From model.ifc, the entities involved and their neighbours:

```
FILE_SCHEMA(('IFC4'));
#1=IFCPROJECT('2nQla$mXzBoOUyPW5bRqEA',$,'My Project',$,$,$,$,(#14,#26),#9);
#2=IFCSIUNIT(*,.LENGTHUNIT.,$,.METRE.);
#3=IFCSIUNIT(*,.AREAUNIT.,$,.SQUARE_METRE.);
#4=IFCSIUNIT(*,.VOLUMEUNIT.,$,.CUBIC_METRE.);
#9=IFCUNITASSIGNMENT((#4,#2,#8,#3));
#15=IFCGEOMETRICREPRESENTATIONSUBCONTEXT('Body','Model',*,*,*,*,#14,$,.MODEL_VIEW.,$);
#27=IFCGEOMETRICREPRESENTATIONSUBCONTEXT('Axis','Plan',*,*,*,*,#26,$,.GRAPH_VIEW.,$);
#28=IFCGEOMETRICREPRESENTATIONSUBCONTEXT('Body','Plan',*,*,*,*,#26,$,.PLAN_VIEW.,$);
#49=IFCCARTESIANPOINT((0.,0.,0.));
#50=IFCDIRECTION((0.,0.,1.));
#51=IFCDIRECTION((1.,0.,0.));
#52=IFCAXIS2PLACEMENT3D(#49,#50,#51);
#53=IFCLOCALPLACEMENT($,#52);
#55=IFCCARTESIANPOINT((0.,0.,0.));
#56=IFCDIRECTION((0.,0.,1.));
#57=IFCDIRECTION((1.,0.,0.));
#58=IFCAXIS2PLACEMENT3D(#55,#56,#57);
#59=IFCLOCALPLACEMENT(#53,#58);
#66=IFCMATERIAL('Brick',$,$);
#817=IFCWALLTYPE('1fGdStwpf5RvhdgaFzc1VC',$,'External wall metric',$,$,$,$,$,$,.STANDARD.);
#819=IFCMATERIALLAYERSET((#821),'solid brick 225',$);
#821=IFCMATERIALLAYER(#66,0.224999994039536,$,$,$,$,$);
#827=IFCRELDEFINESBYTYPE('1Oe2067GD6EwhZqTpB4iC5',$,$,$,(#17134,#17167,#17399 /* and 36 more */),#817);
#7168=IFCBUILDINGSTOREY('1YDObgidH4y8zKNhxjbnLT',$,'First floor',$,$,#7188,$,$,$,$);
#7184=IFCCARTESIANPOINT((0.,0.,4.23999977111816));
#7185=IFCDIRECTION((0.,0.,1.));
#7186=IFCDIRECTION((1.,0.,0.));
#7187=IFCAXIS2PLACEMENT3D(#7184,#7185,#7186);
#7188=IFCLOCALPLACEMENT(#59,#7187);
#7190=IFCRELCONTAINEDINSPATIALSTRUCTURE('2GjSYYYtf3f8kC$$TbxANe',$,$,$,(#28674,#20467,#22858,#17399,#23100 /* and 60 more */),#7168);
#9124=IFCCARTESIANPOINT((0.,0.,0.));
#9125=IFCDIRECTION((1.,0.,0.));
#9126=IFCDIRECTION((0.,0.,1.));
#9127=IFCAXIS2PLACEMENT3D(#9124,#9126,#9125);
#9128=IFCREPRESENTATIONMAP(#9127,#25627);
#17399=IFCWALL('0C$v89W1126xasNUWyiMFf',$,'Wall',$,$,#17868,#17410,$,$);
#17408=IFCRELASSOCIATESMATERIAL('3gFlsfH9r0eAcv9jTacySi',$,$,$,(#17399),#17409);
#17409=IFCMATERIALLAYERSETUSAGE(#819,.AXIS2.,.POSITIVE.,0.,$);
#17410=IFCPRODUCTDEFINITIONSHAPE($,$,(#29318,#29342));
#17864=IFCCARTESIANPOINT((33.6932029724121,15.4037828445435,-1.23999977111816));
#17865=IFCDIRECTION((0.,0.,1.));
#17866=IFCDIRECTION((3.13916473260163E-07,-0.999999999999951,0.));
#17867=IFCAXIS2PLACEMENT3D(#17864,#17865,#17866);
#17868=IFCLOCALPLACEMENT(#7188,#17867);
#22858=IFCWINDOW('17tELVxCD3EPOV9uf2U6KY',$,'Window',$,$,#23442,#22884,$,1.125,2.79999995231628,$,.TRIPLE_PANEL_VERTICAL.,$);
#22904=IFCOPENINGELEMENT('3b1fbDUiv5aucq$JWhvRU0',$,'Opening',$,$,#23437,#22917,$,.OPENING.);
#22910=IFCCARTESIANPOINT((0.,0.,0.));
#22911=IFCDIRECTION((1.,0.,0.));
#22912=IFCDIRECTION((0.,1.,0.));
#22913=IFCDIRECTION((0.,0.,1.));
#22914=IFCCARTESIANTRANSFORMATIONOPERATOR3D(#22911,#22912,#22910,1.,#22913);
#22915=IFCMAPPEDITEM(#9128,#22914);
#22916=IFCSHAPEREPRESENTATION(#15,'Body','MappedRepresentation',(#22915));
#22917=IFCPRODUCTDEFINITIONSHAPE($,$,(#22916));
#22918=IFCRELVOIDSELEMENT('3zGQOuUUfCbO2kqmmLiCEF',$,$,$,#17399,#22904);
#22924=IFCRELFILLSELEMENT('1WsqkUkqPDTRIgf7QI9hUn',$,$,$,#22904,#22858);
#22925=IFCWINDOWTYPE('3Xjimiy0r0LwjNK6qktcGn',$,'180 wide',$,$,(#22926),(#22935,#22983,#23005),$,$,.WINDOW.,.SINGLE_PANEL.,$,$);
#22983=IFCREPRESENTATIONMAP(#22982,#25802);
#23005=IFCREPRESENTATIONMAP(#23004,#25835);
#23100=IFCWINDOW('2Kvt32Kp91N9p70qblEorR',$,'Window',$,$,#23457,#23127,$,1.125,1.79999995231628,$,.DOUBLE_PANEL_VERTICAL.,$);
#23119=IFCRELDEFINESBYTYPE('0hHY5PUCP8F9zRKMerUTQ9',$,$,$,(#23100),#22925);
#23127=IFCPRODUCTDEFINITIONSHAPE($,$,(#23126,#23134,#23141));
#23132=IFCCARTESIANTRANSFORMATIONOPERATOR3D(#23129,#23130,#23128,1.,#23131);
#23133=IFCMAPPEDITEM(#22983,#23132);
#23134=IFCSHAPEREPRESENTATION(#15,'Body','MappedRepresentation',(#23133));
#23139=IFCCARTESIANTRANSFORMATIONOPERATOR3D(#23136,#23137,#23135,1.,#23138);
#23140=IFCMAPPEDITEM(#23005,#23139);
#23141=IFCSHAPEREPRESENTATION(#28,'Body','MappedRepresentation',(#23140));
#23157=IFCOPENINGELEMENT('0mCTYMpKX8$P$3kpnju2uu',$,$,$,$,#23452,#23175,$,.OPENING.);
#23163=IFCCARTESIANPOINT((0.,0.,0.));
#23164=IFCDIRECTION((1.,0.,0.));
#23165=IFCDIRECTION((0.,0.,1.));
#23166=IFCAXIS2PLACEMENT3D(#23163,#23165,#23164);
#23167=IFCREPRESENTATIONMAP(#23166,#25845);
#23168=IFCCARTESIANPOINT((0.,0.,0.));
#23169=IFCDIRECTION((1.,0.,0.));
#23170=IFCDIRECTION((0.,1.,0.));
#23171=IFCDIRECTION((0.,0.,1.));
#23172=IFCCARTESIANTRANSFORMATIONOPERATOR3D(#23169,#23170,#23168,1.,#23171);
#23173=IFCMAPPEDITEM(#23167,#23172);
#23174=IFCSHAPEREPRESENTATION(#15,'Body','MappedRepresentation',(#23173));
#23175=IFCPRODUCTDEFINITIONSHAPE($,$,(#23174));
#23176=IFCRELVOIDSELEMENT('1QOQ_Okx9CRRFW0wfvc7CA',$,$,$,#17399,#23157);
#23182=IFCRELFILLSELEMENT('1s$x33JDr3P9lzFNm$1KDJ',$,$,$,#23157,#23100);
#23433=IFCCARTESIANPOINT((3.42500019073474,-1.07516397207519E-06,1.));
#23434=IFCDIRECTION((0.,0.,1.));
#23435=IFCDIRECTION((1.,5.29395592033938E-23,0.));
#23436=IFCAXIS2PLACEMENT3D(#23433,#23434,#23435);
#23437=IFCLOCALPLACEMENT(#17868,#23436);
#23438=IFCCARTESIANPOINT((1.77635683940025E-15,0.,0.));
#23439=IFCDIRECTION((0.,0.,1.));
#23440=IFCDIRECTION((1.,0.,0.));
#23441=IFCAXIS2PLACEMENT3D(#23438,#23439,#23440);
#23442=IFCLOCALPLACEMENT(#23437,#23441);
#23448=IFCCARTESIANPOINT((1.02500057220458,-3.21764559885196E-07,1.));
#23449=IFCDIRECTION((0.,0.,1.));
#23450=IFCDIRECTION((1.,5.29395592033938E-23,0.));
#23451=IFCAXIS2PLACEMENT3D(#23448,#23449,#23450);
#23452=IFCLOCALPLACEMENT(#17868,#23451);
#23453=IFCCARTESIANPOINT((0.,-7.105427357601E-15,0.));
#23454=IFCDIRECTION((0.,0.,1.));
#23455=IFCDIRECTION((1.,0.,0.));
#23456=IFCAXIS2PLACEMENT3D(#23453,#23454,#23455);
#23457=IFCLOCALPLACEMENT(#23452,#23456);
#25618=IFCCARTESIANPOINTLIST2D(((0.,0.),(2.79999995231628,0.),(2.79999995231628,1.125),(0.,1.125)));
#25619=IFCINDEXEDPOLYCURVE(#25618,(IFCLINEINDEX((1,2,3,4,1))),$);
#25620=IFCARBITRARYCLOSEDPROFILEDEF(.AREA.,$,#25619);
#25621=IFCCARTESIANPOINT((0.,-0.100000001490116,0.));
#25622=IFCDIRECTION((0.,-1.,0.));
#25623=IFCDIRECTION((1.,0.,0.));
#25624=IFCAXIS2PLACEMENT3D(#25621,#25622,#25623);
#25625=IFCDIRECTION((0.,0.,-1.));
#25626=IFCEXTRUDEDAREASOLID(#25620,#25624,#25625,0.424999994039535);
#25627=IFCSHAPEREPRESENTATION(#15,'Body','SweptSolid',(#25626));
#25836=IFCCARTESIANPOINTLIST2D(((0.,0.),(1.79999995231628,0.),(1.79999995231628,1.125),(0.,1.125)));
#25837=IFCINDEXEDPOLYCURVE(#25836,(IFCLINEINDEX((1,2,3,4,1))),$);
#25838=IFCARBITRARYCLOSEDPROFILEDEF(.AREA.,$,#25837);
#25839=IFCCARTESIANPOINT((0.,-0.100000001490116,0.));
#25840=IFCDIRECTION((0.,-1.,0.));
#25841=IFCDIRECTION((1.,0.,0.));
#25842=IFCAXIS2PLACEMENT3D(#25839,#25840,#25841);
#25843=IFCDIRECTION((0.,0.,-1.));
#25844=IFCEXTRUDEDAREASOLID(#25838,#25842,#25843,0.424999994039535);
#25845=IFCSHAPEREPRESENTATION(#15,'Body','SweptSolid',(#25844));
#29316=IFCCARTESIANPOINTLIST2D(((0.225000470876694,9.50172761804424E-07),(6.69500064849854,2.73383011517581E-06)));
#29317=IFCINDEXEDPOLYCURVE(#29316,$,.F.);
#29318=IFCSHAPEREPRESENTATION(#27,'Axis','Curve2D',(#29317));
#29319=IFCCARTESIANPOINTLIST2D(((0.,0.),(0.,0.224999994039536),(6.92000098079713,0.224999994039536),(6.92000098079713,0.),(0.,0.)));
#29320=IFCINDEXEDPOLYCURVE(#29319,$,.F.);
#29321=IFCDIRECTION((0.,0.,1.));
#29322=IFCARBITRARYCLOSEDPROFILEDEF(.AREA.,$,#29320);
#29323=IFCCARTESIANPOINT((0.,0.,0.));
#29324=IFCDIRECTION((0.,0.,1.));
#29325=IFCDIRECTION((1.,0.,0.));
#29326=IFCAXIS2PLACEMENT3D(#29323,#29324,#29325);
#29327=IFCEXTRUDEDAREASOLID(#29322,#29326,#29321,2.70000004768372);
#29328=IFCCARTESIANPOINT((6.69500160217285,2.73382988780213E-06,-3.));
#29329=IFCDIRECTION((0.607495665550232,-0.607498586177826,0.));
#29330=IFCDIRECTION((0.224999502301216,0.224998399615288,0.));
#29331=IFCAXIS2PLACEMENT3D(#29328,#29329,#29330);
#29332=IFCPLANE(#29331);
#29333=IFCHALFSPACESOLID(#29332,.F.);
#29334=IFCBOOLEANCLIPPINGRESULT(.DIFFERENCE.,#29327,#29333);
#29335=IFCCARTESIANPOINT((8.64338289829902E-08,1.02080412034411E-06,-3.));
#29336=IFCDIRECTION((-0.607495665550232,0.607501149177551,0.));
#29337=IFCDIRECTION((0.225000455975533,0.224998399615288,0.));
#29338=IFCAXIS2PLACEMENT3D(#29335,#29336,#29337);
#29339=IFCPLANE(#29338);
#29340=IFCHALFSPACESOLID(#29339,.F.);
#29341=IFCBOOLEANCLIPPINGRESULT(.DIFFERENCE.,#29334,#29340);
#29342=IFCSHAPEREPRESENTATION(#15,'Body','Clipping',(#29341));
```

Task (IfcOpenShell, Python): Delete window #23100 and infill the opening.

```python
import ifcopenshell
import ifcopenshell.api.feature
import ifcopenshell.api.root
import ifcopenshell.geom
import ifcopenshell.util.shape

model = ifcopenshell.open("model.ifc")
settings = ifcopenshell.geom.settings()


def volume(element):
    """Net volume in cubic metres, openings subtracted."""
    shape = ifcopenshell.geom.create_shape(settings, element)
    return ifcopenshell.util.shape.get_volume(shape.geometry)


window = model.by_guid("2Kvt32Kp91N9p70qblEorR")
opening = window.FillsVoids[0].RelatingOpeningElement
wall = opening.VoidsElements[0].RelatingBuildingElement
before = volume(wall)

ifcopenshell.api.root.remove_product(model, product=window)
ifcopenshell.api.feature.remove_feature(model, feature=opening)

after = volume(wall)

print(f"wall volume {before:.3f} -> {after:.3f} m3")

model.write("model-out.ifc")
```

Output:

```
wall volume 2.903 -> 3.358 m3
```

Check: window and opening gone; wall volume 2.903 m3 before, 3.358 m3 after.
